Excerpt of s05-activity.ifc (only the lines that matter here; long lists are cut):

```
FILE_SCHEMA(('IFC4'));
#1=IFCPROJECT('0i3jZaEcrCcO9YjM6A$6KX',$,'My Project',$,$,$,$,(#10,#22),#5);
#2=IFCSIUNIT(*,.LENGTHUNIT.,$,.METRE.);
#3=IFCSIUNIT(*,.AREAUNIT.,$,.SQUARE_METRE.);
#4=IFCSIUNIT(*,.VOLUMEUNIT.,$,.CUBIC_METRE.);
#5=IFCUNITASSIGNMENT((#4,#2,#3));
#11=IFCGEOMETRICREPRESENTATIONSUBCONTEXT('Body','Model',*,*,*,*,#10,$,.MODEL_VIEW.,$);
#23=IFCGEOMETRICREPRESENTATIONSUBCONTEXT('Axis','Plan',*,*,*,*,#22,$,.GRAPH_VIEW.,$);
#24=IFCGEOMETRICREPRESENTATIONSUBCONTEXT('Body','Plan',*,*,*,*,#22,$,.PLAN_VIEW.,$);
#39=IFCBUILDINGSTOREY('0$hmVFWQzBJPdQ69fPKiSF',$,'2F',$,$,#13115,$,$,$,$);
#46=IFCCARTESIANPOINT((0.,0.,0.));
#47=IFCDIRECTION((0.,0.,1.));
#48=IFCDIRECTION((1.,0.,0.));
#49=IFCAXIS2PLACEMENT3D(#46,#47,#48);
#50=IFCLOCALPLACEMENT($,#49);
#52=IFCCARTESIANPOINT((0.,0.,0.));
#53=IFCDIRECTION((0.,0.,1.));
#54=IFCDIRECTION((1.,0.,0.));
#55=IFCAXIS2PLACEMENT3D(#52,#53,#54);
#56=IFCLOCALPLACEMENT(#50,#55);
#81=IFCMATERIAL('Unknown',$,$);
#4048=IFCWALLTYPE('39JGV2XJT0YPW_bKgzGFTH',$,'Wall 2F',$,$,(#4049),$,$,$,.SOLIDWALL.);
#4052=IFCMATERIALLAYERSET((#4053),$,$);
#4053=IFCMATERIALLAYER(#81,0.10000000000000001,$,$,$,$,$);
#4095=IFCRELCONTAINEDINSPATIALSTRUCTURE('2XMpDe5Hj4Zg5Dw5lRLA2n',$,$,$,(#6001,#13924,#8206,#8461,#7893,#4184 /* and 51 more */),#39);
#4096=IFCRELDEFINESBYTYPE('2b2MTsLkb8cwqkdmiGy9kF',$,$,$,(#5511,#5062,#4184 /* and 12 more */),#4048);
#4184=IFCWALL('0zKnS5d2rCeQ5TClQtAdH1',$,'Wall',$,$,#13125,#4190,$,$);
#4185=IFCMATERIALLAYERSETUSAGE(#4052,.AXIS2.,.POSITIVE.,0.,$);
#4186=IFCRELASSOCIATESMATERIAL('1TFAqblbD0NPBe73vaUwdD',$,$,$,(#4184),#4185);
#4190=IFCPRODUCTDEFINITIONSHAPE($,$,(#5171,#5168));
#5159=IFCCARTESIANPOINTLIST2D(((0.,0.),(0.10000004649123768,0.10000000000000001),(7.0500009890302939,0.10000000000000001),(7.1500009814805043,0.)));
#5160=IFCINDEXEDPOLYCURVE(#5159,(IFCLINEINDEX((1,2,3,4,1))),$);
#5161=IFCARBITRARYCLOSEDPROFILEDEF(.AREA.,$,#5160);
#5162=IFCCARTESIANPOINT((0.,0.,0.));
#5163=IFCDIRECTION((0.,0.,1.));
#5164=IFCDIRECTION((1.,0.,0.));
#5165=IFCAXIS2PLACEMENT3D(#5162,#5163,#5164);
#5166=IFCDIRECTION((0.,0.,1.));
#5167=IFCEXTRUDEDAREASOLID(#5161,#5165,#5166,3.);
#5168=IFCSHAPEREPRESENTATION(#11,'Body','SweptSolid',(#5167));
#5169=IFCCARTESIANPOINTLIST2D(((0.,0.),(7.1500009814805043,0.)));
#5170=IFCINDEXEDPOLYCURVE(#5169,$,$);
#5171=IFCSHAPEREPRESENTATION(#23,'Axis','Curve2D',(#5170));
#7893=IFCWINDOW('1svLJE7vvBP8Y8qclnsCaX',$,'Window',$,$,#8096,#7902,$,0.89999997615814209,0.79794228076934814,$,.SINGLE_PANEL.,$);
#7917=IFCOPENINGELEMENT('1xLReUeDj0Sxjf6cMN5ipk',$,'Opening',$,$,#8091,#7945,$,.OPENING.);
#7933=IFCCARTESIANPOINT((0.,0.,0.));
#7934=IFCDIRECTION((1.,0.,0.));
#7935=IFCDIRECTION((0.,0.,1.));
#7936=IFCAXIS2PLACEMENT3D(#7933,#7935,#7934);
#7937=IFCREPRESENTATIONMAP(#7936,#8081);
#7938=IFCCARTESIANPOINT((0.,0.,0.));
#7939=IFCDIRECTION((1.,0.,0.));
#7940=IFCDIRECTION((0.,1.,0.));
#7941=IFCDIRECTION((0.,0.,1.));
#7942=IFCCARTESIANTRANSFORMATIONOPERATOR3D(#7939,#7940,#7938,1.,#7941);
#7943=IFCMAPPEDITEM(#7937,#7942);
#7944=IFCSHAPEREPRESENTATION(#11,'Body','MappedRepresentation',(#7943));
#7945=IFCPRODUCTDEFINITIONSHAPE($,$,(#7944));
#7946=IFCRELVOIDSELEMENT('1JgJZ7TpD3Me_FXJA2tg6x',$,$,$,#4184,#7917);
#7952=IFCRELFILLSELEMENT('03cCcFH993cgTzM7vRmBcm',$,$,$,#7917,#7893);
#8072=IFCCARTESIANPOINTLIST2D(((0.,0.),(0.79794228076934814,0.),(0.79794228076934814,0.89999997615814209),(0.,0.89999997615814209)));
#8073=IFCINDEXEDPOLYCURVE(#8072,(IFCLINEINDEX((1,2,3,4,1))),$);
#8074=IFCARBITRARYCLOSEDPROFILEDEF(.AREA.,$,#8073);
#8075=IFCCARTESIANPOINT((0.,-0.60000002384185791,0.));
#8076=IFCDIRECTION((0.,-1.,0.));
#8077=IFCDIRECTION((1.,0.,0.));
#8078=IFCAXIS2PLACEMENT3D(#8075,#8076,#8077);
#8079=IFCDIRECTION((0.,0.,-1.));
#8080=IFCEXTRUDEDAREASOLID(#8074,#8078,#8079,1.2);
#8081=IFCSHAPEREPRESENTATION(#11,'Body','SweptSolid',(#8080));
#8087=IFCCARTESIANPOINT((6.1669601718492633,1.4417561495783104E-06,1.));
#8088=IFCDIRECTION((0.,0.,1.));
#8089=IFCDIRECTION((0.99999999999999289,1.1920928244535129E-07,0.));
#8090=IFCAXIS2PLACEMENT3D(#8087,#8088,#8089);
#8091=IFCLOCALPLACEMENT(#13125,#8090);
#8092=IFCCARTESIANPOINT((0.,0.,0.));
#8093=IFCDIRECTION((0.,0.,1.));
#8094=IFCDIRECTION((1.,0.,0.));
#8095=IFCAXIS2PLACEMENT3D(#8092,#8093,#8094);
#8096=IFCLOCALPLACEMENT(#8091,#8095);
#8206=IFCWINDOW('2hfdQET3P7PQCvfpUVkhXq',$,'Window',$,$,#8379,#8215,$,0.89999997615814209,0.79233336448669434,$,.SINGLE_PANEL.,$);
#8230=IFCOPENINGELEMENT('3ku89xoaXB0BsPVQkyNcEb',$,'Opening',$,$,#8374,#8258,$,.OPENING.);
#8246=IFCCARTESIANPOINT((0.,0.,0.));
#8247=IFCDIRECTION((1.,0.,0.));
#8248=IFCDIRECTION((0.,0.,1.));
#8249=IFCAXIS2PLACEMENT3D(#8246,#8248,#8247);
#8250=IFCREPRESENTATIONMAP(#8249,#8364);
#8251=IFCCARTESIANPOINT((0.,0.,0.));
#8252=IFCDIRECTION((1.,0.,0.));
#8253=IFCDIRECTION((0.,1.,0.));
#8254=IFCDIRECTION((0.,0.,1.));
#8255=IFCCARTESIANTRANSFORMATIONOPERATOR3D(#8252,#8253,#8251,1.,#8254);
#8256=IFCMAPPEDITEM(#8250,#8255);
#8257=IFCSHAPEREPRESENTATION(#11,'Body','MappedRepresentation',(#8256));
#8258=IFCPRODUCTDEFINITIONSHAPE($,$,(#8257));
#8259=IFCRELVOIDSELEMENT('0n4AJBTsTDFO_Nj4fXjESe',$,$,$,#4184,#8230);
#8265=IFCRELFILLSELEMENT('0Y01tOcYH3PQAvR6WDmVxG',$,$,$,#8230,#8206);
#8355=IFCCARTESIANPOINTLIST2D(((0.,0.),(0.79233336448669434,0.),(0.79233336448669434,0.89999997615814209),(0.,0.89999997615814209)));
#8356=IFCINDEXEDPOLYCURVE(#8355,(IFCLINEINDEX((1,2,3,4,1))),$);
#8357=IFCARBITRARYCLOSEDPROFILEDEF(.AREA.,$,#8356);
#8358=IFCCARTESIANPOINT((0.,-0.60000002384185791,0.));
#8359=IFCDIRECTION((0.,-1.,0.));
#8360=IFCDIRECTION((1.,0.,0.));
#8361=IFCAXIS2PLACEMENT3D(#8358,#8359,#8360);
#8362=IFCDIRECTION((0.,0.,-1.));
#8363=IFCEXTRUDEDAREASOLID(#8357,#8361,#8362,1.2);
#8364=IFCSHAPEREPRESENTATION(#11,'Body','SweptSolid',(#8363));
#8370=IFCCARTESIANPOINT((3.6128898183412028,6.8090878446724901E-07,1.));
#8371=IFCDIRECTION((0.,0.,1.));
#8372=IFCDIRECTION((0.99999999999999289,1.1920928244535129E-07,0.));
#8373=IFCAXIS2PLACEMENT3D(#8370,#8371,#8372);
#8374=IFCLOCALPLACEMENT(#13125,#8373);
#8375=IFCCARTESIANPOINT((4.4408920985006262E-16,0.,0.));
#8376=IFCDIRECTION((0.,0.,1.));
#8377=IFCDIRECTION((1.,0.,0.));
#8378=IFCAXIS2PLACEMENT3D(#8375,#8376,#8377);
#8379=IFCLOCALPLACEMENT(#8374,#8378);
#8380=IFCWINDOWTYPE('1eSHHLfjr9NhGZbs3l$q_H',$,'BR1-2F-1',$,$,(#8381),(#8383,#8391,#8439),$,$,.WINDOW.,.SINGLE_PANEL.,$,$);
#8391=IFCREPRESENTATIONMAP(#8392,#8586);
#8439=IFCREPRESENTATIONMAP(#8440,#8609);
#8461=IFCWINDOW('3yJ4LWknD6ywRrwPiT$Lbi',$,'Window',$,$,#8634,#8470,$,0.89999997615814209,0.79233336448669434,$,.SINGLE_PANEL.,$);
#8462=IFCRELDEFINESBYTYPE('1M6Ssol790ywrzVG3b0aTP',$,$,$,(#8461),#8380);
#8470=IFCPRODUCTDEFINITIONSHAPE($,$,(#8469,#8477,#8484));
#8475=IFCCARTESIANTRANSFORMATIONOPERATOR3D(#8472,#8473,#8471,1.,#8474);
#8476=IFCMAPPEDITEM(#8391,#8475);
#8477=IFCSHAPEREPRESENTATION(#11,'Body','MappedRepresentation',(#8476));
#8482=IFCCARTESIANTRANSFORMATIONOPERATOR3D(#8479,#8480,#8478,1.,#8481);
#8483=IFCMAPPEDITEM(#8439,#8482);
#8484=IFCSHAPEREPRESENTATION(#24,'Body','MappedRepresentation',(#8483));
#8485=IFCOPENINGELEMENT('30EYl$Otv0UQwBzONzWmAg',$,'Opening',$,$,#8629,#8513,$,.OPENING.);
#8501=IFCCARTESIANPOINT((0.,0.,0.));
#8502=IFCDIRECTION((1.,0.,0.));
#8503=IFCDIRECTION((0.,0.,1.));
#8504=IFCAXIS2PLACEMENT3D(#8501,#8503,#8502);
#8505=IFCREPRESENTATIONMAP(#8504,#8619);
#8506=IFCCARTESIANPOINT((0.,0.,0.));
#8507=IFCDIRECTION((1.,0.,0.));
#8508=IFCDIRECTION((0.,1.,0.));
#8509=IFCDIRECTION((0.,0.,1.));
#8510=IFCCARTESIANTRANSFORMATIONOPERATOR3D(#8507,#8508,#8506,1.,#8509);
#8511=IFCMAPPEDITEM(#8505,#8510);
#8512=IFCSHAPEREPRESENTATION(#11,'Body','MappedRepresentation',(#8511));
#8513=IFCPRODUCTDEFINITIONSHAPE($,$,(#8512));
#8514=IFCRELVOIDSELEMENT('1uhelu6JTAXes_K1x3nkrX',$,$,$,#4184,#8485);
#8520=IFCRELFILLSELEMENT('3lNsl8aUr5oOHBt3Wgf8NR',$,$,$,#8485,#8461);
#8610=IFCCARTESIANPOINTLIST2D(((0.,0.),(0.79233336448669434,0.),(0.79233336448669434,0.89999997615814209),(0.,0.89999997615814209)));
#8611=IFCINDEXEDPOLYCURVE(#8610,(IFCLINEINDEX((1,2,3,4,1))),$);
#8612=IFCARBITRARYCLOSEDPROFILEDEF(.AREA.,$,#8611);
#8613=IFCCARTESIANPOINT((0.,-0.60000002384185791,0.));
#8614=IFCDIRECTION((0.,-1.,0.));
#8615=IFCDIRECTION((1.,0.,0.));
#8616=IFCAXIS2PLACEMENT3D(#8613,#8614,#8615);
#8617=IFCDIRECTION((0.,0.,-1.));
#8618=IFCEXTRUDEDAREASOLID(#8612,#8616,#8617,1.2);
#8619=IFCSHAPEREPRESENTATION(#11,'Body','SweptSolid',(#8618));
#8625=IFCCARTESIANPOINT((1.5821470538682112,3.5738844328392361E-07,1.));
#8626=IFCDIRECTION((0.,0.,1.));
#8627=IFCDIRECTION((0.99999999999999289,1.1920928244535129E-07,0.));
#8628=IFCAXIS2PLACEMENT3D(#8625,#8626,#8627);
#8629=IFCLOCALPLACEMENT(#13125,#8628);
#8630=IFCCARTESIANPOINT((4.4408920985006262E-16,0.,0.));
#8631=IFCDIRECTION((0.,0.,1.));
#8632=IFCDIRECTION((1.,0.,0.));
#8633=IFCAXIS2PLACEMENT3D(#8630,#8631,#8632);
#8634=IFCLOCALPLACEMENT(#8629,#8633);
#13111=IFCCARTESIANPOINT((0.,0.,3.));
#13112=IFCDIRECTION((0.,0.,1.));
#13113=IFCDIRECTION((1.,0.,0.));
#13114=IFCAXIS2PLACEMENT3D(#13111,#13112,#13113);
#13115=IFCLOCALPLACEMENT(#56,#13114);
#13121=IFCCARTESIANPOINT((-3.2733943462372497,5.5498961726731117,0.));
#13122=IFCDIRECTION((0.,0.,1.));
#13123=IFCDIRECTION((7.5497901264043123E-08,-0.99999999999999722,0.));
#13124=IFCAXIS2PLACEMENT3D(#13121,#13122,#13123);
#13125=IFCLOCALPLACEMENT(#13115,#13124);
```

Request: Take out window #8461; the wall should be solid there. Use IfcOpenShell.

```python
import ifcopenshell
import ifcopenshell.api.feature
import ifcopenshell.api.root
import ifcopenshell.geom
import ifcopenshell.util.shape

model = ifcopenshell.open("s05-activity.ifc")
settings = ifcopenshell.geom.settings()


def volume(element):
    """Net volume in cubic metres, openings subtracted."""
    shape = ifcopenshell.geom.create_shape(settings, element)
    return ifcopenshell.util.shape.get_volume(shape.geometry)


window = model.by_guid("3yJ4LWknD6ywRrwPiT$Lbi")
opening = window.FillsVoids[0].RelatingOpeningElement
wall = opening.VoidsElements[0].RelatingBuildingElement
before = volume(wall)

ifcopenshell.api.root.remove_product(model, product=window)
ifcopenshell.api.feature.remove_feature(model, feature=opening)

after = volume(wall)

print(f"wall volume {before:.3f} -> {after:.3f} m3")

model.write("s05-activity_edited.ifc")
```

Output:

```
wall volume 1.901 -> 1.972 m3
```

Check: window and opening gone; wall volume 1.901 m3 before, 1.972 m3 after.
